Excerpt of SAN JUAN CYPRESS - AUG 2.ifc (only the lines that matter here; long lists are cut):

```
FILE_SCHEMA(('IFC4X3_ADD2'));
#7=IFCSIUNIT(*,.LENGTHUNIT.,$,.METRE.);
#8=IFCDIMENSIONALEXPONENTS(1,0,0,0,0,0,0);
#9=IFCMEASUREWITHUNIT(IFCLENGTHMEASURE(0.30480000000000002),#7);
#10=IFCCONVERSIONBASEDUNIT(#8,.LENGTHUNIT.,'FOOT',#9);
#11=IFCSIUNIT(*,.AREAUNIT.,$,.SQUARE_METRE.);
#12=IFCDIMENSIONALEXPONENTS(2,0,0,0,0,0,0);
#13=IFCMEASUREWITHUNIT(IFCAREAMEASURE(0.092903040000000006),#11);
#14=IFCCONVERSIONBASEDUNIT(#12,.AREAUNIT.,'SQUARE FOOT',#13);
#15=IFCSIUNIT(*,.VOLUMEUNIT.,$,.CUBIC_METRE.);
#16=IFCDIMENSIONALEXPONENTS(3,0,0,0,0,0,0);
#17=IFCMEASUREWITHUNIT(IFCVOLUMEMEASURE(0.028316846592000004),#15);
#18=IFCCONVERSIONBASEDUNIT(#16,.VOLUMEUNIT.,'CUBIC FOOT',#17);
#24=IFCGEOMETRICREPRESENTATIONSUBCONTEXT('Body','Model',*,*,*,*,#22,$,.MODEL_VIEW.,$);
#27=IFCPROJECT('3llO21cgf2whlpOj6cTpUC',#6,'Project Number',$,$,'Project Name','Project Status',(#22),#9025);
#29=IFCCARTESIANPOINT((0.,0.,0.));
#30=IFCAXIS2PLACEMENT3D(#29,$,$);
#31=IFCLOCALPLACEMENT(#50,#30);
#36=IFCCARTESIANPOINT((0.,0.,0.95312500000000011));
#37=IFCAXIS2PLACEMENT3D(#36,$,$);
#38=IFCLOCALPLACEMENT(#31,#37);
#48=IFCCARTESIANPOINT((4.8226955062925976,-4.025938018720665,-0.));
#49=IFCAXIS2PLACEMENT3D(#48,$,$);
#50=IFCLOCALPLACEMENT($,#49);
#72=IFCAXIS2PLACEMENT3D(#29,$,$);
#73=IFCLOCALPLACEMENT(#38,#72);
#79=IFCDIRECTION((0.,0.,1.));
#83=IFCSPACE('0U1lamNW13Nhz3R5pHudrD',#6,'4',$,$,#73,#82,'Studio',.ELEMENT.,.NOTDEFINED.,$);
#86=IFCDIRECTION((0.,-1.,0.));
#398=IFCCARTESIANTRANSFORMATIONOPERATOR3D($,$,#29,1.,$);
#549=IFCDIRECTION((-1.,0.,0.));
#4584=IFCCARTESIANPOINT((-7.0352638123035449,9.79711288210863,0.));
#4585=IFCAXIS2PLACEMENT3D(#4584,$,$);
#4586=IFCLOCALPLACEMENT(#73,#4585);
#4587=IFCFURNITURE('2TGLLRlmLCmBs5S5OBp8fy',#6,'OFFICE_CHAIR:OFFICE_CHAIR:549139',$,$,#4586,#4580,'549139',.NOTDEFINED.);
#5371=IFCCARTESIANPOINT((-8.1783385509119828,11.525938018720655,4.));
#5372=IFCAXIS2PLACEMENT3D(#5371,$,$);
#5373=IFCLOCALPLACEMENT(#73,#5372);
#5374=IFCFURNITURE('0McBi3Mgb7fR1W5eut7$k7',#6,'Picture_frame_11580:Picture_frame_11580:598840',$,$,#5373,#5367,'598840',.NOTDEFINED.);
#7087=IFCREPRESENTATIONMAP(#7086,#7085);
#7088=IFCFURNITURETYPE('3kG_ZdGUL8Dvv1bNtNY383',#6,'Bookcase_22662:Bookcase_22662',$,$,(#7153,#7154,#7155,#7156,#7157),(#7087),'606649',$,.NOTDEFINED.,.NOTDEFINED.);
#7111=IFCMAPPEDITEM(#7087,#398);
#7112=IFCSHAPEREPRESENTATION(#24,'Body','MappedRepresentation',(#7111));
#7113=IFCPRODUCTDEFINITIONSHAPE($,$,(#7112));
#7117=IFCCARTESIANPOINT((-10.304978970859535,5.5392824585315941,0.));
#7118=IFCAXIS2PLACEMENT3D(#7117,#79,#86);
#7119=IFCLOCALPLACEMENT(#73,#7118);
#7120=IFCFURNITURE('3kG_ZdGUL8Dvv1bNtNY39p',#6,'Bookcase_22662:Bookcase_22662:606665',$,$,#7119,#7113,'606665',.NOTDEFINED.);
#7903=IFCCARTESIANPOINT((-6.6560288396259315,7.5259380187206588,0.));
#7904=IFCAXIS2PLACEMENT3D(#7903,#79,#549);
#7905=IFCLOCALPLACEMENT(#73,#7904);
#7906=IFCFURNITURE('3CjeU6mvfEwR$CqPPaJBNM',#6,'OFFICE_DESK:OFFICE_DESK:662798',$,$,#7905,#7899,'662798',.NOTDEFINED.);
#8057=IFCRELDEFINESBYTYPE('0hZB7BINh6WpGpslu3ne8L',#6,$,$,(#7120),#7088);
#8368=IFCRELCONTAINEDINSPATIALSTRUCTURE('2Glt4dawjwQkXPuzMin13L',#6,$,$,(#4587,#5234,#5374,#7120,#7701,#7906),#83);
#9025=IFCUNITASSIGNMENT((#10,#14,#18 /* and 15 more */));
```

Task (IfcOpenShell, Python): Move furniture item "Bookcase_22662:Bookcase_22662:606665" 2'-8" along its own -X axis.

```python
import ifcopenshell
import ifcopenshell.api.geometry
import ifcopenshell.util.placement
import ifcopenshell.util.unit

model = ifcopenshell.open("SAN JUAN CYPRESS - AUG 2.ifc")
unit_scale = ifcopenshell.util.unit.calculate_unit_scale(model)

item = model.by_guid("3kG_ZdGUL8Dvv1bNtNY39p")
matrix = ifcopenshell.util.placement.get_local_placement(item.ObjectPlacement)
matrix[:3, 3] -= matrix[:3, 0] * 32 * 0.0254 / unit_scale
ifcopenshell.api.geometry.edit_object_placement(model, product=item, matrix=matrix, is_si=False)

print(ifcopenshell.util.placement.get_local_placement(item.ObjectPlacement).round(3) + 0.0)

model.write("SAN JUAN CYPRESS - AUG 2_edited.ifc")
```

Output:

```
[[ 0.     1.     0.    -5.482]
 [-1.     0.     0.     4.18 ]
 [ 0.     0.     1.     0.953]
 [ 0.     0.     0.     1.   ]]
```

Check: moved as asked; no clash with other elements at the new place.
